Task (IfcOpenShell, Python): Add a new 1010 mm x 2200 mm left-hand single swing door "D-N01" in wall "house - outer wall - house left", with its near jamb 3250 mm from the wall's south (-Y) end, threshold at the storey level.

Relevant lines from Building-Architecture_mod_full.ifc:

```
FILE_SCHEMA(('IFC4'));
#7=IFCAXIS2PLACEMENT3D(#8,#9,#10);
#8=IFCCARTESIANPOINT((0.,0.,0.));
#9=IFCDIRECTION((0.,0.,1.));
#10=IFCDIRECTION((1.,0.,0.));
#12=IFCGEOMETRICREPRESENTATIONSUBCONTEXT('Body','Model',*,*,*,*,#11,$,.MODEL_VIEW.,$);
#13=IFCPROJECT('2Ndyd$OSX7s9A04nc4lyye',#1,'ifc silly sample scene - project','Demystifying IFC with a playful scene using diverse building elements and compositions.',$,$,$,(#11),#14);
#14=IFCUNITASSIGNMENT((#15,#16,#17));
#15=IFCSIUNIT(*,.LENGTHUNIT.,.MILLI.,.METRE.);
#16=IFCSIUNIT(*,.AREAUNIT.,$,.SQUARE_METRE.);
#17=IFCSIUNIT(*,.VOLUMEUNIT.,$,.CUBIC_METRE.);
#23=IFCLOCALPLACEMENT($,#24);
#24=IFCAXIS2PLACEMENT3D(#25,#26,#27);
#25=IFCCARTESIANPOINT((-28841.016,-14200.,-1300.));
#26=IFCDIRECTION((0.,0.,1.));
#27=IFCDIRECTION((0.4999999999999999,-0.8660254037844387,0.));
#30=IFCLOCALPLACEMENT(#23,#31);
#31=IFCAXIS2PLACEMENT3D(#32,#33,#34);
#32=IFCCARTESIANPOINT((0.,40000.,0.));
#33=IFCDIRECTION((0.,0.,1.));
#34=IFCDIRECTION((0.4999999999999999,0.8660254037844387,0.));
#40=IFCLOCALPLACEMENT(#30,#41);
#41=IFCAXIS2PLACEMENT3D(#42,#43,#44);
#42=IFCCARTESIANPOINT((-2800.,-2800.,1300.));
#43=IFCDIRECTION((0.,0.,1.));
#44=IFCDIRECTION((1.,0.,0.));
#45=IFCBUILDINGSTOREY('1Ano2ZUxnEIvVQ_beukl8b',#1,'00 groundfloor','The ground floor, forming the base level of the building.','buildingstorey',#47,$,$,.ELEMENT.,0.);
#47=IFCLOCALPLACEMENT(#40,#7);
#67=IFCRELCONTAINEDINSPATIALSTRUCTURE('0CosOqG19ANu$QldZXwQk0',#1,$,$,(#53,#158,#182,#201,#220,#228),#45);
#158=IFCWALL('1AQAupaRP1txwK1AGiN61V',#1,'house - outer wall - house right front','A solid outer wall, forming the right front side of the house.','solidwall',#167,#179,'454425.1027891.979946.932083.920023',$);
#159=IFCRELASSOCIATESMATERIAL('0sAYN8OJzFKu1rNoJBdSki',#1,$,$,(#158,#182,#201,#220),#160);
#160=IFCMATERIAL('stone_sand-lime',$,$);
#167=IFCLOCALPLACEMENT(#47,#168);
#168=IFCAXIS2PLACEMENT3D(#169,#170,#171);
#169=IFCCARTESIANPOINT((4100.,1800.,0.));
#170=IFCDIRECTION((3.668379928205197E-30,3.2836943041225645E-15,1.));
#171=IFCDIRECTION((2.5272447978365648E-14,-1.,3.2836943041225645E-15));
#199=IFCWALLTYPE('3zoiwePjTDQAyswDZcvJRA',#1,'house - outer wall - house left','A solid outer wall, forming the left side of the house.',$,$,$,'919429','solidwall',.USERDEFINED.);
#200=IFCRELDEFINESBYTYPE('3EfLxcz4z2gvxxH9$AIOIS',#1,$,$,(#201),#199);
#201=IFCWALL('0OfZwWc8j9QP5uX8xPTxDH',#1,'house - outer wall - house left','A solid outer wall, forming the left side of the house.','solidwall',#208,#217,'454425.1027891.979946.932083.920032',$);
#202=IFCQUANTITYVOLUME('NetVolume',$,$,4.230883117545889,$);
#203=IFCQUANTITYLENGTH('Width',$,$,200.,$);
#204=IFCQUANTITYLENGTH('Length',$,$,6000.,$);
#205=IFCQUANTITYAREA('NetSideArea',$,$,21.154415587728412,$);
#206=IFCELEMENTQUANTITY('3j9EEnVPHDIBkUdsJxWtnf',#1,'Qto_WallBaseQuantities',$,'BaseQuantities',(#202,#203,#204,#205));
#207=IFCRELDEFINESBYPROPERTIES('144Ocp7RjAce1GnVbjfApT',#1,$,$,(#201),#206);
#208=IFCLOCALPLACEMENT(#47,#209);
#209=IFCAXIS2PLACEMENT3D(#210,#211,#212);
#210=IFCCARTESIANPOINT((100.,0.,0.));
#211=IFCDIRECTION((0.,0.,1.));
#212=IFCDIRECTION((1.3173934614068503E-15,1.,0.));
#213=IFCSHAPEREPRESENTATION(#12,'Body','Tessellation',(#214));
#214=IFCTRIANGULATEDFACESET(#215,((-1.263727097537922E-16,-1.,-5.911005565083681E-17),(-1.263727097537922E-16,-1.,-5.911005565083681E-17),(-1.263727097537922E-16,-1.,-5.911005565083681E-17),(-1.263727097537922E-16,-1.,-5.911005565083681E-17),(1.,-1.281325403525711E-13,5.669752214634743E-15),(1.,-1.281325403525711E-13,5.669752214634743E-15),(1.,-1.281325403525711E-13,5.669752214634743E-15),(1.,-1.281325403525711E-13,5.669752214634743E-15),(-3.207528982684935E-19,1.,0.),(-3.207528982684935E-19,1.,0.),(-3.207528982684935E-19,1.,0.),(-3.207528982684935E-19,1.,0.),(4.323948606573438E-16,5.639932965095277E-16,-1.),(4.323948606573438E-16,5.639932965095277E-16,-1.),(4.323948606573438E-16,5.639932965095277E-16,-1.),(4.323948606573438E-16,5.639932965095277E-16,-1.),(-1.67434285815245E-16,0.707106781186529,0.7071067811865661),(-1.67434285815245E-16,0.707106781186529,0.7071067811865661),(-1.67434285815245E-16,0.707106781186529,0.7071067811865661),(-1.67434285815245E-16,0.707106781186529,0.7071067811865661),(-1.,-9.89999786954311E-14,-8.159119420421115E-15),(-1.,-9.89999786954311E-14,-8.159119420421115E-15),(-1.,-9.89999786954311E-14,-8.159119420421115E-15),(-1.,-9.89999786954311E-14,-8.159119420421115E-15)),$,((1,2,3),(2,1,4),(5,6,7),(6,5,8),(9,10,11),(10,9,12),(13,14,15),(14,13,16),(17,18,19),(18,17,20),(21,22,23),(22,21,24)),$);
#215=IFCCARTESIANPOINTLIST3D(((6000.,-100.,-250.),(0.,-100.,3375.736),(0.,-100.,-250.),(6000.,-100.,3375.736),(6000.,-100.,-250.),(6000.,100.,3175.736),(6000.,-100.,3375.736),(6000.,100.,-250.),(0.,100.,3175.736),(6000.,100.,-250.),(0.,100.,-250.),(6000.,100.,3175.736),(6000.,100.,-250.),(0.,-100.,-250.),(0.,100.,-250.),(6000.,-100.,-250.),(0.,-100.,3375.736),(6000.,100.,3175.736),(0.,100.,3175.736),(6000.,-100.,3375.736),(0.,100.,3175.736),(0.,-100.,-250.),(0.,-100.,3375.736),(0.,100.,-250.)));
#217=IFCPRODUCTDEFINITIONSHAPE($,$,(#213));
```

```python
import numpy as np
import ifcopenshell
import ifcopenshell.api.feature
import ifcopenshell.api.geometry
import ifcopenshell.api.pset
import ifcopenshell.api.root
import ifcopenshell.api.spatial
import ifcopenshell.geom
import ifcopenshell.util.element
import ifcopenshell.util.placement
import ifcopenshell.util.representation
import ifcopenshell.util.shape
import ifcopenshell.util.unit

model = ifcopenshell.open("Building-Architecture_mod_full.ifc")
unit_scale = ifcopenshell.util.unit.calculate_unit_scale(model)
area_scale = ifcopenshell.util.unit.calculate_unit_scale(model, "AREAUNIT")
volume_scale = ifcopenshell.util.unit.calculate_unit_scale(model, "VOLUMEUNIT")
settings = ifcopenshell.geom.settings()


def volume(element):
    """Net volume in cubic metres, openings subtracted."""
    shape = ifcopenshell.geom.create_shape(settings, element)
    return ifcopenshell.util.shape.get_volume(shape.geometry)


wall = model.by_guid("0OfZwWc8j9QP5uX8xPTxDH")
storey = ifcopenshell.util.element.get_container(wall, ifc_class="IfcBuildingStorey")
context = ifcopenshell.util.representation.get_context(model, "Model", "Body", "MODEL_VIEW")
before = volume(wall)

width, height, from_end, sill = 1.01, 2.2, 3.25, 0.0  # metres

# The wall runs along its own X axis, and the end named is its -X end.
wall_shape = ifcopenshell.geom.create_shape(settings, wall)
x, y, z = ifcopenshell.util.shape.get_vertices(wall_shape.geometry).T
start = x.min() + from_end
face, thickness = float(y.min()), float(y.max() - y.min())
wall_matrix = ifcopenshell.util.placement.get_local_placement(wall.ObjectPlacement)
level = ifcopenshell.util.placement.get_local_placement(storey.ObjectPlacement)[2, 3]


def in_wall(x, y):
    """Placement at x, y metres in the wall's axes, at sill height."""
    matrix = wall_matrix.copy()
    matrix[:, 3] = wall_matrix @ np.array([x / unit_scale, y / unit_scale, 0.0, 1.0])
    matrix[2, 3] = level + sill / unit_scale
    return matrix


# Opening: a box that overshoots both wall faces by 50 mm.
opening = ifcopenshell.api.root.create_entity(model, ifc_class="IfcOpeningElement", predefined_type="OPENING")
box = ifcopenshell.api.geometry.add_wall_representation(
    model, context=context, length=width, height=height, thickness=thickness + 0.1
)
ifcopenshell.api.geometry.assign_representation(model, product=opening, representation=box)
ifcopenshell.api.geometry.edit_object_placement(model, product=opening, matrix=in_wall(start, face - 0.05), is_si=False)
ifcopenshell.api.feature.add_feature(model, feature=opening, element=wall)

door = ifcopenshell.api.root.create_entity(model, ifc_class="IfcDoor", name="D-N01", predefined_type="DOOR")
door.OverallWidth, door.OverallHeight = width / unit_scale, height / unit_scale
door.OperationType = "SINGLE_SWING_LEFT"
body = ifcopenshell.api.geometry.add_door_representation(
    model,
    context=context,
    overall_width=door.OverallWidth,
    overall_height=door.OverallHeight,
    operation_type="SINGLE_SWING_LEFT",
    lining_properties={"LiningDepth": thickness / unit_scale, "ThresholdDepth": thickness / unit_scale},
)
ifcopenshell.api.geometry.assign_representation(model, product=door, representation=body)
ifcopenshell.api.spatial.assign_container(model, products=[door], relating_structure=storey)
ifcopenshell.api.feature.add_filling(model, opening=opening, element=door)

# The lining spans the wall, so the door starts at the wall face.
ifcopenshell.api.geometry.edit_object_placement(model, product=door, matrix=in_wall(start, face), is_si=False)

after = volume(wall)

# Update the wall's stored quantities.
qto = model.by_id(ifcopenshell.util.element.get_pset(wall, "Qto_WallBaseQuantities", should_inherit=False)["id"])
ifcopenshell.api.pset.edit_qto(model, qto=qto, properties={
    "NetVolume": after / volume_scale,
    "NetSideArea": after / thickness / area_scale,
})

print(f"wall volume {before:.3f} -> {after:.3f} m3")

model.write("Building-Architecture_mod_full_v2.ifc")
```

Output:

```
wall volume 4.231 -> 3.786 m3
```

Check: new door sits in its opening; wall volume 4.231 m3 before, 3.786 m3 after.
